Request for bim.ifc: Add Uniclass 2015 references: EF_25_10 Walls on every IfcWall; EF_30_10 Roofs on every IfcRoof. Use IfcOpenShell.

First a look at what the model holds.

```python
import ifcopenshell

model = ifcopenshell.open("bim.ifc")
print(model.schema)
print("classifications:", [c.Name for c in model.by_type("IfcClassification")])
for ifc_class in ("IfcDoor", "IfcRoof", "IfcStair", "IfcWall", "IfcWindow"):
    print(ifc_class, len(model.by_type(ifc_class)))
```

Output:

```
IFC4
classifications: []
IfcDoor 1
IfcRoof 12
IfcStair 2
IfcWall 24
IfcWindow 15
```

```python
import ifcopenshell
import ifcopenshell.api.classification

model = ifcopenshell.open("bim.ifc")

system = ifcopenshell.api.classification.add_classification(model, classification="Uniclass 2015")

codes = {
    "IfcWall": ("EF_25_10", "Walls"),
    "IfcRoof": ("EF_30_10", "Roofs"),
}
for ifc_class, (code, name) in codes.items():
    products = model.by_type(ifc_class)
    ifcopenshell.api.classification.add_reference(
        model, products=products, classification=system, identification=code, name=name
    )
    print(code, len(products))

model.write("bim_edited.ifc")
```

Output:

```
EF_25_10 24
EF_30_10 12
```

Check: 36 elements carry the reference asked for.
